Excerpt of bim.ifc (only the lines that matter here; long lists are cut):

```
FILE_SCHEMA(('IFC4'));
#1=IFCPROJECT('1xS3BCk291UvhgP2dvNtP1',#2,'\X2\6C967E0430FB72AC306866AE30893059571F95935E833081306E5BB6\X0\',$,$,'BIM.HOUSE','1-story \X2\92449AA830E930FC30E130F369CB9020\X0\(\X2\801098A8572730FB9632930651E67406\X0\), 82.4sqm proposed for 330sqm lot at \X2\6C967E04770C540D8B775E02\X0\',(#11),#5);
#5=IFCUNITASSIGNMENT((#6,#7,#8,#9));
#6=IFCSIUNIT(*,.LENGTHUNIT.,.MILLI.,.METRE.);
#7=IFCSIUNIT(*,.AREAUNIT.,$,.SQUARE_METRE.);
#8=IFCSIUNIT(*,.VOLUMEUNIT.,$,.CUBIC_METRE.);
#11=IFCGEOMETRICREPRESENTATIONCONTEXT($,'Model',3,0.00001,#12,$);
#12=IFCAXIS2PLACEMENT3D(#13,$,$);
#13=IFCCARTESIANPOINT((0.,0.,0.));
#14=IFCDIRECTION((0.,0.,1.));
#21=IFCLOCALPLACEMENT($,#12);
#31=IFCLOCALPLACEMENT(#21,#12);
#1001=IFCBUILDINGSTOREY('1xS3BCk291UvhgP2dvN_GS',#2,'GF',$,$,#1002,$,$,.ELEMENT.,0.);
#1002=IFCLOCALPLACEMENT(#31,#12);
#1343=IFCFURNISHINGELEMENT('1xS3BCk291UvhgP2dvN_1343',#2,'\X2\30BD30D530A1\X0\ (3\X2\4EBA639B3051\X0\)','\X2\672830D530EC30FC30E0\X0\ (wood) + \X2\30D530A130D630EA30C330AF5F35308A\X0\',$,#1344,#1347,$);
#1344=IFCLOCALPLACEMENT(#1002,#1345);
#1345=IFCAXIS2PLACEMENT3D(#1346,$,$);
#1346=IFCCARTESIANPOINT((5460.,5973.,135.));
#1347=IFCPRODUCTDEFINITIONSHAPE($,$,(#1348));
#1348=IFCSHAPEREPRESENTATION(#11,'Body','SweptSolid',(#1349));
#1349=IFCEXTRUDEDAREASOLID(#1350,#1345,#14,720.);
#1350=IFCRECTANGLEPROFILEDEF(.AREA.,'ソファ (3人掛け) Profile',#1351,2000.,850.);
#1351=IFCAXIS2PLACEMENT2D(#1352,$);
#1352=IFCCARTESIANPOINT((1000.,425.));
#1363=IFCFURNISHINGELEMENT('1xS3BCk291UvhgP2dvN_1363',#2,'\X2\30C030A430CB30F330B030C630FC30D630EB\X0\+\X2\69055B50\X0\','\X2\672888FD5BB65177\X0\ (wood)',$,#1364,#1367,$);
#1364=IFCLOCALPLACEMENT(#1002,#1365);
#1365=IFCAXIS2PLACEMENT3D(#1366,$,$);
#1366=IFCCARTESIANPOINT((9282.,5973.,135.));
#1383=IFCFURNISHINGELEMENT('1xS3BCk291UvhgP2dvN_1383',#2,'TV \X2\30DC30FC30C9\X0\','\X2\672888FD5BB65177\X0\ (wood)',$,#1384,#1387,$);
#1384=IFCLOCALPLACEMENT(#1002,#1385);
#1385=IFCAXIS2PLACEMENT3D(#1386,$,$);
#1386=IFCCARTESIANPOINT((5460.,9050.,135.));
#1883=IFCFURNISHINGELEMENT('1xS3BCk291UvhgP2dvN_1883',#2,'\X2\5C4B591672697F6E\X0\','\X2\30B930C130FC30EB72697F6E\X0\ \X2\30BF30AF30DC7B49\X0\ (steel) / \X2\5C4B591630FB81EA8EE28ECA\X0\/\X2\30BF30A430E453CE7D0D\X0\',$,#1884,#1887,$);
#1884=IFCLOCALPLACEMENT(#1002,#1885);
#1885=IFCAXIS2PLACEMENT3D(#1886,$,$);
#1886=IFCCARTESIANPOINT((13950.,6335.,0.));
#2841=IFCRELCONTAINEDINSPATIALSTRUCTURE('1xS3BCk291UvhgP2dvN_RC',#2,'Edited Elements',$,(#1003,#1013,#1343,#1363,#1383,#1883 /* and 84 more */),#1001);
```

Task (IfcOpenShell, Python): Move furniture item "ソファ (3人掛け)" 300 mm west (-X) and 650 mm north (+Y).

```python
import ifcopenshell
import ifcopenshell.api.geometry
import ifcopenshell.util.placement
import ifcopenshell.util.unit

model = ifcopenshell.open("bim.ifc")
unit_scale = ifcopenshell.util.unit.calculate_unit_scale(model)

item = model.by_id(1343)
matrix = ifcopenshell.util.placement.get_local_placement(item.ObjectPlacement)
matrix[0, 3] -= 0.3 / unit_scale
matrix[1, 3] += 0.65 / unit_scale
ifcopenshell.api.geometry.edit_object_placement(model, product=item, matrix=matrix, is_si=False)

print(ifcopenshell.util.placement.get_local_placement(item.ObjectPlacement).round(3) + 0.0)

model.write("bim_rev.ifc")
```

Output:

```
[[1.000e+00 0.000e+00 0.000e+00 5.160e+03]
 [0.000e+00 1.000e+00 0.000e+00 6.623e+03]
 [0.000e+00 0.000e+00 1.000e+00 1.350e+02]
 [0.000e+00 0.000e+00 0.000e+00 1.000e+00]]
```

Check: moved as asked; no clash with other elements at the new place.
